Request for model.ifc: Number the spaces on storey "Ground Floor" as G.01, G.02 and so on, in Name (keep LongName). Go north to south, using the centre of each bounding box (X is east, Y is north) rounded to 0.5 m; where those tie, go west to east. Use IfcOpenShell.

First a look at what the model holds.

```python
import ifcopenshell
import ifcopenshell.util.element
import ifcopenshell.util.placement

model = ifcopenshell.open("model.ifc")
print(model.schema)
storey = next(s for s in model.by_type("IfcBuildingStorey") if s.Name == "Ground Floor")
spaces = [e for e in ifcopenshell.util.element.get_decomposition(storey) if e.is_a("IfcSpace")]
for e in sorted(spaces, key=lambda e: e.id()):
    origin = ifcopenshell.util.placement.get_local_placement(e.ObjectPlacement)[:3, 3]
    print(e.id(), e.Name, e.LongName, origin.round(2) + 0.0, sep=" | ")
```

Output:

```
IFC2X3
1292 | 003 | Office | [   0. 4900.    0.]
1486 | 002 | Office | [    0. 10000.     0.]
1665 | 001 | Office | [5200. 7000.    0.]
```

```python
import ifcopenshell
import ifcopenshell.geom
import ifcopenshell.util.element
import ifcopenshell.util.shape

model = ifcopenshell.open("model.ifc")
settings = ifcopenshell.geom.settings()
settings.set("use-world-coords", True)


def centre(element):
    shape = ifcopenshell.geom.create_shape(settings, element)
    return ifcopenshell.util.shape.get_bbox_centroid(shape.geometry)


storey = next(s for s in model.by_type("IfcBuildingStorey") if s.Name == "Ground Floor")
spaces = [e for e in ifcopenshell.util.element.get_decomposition(storey) if e.is_a("IfcSpace")]

# Insertion points can sit at a corner or the storey origin, so sort by the geometry (in metres).
centres = {e: centre(e) for e in spaces}
spaces.sort(key=lambda e: (-round(centres[e][1] / 0.5), centres[e][0]))

for i, e in enumerate(spaces, start=1):
    number = f"G.{i:02d}"
    e.Name = number
    print(e.id(), number)

model.write("model_edited.ifc")
```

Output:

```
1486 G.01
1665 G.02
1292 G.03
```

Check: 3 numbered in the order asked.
